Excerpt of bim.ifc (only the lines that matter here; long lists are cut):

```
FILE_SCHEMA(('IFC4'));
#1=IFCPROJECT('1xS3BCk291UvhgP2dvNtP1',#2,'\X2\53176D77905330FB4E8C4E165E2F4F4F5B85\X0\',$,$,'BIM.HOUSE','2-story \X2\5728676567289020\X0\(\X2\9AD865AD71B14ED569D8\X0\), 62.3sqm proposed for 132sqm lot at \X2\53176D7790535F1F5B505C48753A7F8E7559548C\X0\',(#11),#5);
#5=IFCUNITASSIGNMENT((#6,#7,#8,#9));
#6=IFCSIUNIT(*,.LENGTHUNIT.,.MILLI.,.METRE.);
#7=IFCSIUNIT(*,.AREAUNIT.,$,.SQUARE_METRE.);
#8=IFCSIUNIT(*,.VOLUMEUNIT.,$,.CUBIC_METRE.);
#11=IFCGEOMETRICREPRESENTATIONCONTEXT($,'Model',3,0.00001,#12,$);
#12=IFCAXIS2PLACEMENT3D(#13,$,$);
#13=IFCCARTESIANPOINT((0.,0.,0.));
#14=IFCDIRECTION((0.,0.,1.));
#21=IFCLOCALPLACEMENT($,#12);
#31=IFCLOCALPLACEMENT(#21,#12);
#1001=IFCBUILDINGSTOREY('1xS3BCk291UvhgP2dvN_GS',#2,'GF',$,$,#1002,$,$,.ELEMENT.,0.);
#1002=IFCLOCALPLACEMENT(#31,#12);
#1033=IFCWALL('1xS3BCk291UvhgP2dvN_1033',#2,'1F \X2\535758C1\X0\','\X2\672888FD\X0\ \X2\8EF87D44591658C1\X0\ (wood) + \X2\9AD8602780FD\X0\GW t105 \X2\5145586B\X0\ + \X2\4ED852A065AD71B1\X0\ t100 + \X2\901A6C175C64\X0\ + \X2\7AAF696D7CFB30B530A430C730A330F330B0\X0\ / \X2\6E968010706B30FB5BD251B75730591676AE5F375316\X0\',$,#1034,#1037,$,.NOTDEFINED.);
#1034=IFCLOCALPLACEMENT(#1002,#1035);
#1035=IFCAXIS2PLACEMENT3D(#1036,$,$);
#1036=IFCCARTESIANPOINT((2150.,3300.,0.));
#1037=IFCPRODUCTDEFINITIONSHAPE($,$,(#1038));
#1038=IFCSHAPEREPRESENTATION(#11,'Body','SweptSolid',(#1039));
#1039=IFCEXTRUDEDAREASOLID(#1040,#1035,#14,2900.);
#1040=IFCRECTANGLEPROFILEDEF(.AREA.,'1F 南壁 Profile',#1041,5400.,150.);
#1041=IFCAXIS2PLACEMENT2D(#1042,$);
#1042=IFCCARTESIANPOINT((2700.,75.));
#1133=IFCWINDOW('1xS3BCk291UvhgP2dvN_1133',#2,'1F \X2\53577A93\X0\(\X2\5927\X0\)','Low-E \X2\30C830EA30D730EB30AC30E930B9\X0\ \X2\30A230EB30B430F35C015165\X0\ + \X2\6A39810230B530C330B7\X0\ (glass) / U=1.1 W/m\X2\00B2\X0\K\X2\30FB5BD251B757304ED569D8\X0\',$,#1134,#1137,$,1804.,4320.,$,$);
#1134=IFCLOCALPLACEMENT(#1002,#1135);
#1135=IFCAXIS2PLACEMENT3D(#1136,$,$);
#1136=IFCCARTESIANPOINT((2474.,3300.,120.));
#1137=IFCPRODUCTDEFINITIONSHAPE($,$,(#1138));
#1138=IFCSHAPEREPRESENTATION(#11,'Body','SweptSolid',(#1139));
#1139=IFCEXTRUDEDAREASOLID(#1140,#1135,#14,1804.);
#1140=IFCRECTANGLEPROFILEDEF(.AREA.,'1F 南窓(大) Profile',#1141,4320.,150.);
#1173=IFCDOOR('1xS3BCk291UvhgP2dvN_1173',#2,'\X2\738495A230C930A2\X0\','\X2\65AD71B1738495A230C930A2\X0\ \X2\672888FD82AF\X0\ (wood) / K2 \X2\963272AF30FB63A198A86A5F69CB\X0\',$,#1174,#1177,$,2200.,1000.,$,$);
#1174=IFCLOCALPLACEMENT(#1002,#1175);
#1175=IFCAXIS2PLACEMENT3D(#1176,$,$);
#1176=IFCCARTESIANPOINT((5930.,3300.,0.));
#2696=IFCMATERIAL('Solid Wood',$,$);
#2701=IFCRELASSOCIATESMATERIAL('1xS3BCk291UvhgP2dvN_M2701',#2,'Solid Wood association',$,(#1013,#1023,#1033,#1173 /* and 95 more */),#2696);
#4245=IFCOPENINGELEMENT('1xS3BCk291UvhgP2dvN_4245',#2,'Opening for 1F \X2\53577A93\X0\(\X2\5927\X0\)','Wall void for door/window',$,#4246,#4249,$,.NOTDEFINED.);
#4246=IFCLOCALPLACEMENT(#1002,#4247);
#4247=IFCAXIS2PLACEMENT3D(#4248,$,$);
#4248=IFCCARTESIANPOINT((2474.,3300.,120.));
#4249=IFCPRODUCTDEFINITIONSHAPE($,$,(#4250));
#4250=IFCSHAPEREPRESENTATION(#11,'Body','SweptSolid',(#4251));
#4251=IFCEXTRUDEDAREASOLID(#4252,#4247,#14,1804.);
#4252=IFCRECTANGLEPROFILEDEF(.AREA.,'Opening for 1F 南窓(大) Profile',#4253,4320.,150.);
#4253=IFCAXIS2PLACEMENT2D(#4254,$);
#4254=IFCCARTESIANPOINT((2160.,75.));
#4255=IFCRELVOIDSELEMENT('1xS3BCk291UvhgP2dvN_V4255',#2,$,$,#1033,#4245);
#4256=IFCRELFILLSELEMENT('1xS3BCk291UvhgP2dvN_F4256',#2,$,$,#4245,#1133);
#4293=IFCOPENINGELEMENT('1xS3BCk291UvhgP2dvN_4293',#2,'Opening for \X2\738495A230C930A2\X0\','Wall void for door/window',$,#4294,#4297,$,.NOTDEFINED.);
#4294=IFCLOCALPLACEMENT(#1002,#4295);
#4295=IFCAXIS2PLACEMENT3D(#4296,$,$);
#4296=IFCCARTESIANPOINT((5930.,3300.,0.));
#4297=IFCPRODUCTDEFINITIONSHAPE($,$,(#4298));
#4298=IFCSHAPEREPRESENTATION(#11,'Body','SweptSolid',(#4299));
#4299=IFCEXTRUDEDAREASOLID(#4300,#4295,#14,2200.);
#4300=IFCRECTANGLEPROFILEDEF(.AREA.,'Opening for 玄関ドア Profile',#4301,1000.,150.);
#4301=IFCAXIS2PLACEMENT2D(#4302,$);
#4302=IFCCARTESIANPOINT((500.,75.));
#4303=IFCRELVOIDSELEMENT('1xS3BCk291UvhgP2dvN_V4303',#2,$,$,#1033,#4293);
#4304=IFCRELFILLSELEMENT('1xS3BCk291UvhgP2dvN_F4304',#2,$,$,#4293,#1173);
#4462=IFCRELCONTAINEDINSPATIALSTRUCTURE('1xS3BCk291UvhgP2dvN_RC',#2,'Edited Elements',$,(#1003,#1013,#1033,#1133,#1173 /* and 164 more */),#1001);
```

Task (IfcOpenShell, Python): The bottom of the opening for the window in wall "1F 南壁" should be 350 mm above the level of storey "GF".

```python
import numpy as np
import ifcopenshell
import ifcopenshell.api.geometry
import ifcopenshell.geom
import ifcopenshell.util.element
import ifcopenshell.util.placement
import ifcopenshell.util.shape
import ifcopenshell.util.unit

model = ifcopenshell.open("bim.ifc")
unit_scale = ifcopenshell.util.unit.calculate_unit_scale(model)

window = model.by_id(1133)
opening = window.FillsVoids[0].RelatingOpeningElement
storey = ifcopenshell.util.element.get_container(window, ifc_class="IfcBuildingStorey")
level = ifcopenshell.util.placement.get_local_placement(storey.ObjectPlacement)[2, 3]

# The opening's origin need not be at the sill, so measure its lowest point.
shape = ifcopenshell.geom.create_shape(ifcopenshell.geom.settings(), opening)
bottom = ifcopenshell.util.shape.get_shape_bottom_elevation(shape, shape.geometry) / unit_scale
dz = level + 0.35 / unit_scale - bottom

shift = np.array([0.0, 0.0, dz])
# The window is not placed relative to its opening, so move both.
for product in (opening, window):
    matrix = ifcopenshell.util.placement.get_local_placement(product.ObjectPlacement)
    matrix[:3, 3] += shift
    ifcopenshell.api.geometry.edit_object_placement(model, product=product, matrix=matrix, is_si=False)

print(f"moved by {dz * unit_scale:+.3f} m")

model.write("bim_rev.ifc")
```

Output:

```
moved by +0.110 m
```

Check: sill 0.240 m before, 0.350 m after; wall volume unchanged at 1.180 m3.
